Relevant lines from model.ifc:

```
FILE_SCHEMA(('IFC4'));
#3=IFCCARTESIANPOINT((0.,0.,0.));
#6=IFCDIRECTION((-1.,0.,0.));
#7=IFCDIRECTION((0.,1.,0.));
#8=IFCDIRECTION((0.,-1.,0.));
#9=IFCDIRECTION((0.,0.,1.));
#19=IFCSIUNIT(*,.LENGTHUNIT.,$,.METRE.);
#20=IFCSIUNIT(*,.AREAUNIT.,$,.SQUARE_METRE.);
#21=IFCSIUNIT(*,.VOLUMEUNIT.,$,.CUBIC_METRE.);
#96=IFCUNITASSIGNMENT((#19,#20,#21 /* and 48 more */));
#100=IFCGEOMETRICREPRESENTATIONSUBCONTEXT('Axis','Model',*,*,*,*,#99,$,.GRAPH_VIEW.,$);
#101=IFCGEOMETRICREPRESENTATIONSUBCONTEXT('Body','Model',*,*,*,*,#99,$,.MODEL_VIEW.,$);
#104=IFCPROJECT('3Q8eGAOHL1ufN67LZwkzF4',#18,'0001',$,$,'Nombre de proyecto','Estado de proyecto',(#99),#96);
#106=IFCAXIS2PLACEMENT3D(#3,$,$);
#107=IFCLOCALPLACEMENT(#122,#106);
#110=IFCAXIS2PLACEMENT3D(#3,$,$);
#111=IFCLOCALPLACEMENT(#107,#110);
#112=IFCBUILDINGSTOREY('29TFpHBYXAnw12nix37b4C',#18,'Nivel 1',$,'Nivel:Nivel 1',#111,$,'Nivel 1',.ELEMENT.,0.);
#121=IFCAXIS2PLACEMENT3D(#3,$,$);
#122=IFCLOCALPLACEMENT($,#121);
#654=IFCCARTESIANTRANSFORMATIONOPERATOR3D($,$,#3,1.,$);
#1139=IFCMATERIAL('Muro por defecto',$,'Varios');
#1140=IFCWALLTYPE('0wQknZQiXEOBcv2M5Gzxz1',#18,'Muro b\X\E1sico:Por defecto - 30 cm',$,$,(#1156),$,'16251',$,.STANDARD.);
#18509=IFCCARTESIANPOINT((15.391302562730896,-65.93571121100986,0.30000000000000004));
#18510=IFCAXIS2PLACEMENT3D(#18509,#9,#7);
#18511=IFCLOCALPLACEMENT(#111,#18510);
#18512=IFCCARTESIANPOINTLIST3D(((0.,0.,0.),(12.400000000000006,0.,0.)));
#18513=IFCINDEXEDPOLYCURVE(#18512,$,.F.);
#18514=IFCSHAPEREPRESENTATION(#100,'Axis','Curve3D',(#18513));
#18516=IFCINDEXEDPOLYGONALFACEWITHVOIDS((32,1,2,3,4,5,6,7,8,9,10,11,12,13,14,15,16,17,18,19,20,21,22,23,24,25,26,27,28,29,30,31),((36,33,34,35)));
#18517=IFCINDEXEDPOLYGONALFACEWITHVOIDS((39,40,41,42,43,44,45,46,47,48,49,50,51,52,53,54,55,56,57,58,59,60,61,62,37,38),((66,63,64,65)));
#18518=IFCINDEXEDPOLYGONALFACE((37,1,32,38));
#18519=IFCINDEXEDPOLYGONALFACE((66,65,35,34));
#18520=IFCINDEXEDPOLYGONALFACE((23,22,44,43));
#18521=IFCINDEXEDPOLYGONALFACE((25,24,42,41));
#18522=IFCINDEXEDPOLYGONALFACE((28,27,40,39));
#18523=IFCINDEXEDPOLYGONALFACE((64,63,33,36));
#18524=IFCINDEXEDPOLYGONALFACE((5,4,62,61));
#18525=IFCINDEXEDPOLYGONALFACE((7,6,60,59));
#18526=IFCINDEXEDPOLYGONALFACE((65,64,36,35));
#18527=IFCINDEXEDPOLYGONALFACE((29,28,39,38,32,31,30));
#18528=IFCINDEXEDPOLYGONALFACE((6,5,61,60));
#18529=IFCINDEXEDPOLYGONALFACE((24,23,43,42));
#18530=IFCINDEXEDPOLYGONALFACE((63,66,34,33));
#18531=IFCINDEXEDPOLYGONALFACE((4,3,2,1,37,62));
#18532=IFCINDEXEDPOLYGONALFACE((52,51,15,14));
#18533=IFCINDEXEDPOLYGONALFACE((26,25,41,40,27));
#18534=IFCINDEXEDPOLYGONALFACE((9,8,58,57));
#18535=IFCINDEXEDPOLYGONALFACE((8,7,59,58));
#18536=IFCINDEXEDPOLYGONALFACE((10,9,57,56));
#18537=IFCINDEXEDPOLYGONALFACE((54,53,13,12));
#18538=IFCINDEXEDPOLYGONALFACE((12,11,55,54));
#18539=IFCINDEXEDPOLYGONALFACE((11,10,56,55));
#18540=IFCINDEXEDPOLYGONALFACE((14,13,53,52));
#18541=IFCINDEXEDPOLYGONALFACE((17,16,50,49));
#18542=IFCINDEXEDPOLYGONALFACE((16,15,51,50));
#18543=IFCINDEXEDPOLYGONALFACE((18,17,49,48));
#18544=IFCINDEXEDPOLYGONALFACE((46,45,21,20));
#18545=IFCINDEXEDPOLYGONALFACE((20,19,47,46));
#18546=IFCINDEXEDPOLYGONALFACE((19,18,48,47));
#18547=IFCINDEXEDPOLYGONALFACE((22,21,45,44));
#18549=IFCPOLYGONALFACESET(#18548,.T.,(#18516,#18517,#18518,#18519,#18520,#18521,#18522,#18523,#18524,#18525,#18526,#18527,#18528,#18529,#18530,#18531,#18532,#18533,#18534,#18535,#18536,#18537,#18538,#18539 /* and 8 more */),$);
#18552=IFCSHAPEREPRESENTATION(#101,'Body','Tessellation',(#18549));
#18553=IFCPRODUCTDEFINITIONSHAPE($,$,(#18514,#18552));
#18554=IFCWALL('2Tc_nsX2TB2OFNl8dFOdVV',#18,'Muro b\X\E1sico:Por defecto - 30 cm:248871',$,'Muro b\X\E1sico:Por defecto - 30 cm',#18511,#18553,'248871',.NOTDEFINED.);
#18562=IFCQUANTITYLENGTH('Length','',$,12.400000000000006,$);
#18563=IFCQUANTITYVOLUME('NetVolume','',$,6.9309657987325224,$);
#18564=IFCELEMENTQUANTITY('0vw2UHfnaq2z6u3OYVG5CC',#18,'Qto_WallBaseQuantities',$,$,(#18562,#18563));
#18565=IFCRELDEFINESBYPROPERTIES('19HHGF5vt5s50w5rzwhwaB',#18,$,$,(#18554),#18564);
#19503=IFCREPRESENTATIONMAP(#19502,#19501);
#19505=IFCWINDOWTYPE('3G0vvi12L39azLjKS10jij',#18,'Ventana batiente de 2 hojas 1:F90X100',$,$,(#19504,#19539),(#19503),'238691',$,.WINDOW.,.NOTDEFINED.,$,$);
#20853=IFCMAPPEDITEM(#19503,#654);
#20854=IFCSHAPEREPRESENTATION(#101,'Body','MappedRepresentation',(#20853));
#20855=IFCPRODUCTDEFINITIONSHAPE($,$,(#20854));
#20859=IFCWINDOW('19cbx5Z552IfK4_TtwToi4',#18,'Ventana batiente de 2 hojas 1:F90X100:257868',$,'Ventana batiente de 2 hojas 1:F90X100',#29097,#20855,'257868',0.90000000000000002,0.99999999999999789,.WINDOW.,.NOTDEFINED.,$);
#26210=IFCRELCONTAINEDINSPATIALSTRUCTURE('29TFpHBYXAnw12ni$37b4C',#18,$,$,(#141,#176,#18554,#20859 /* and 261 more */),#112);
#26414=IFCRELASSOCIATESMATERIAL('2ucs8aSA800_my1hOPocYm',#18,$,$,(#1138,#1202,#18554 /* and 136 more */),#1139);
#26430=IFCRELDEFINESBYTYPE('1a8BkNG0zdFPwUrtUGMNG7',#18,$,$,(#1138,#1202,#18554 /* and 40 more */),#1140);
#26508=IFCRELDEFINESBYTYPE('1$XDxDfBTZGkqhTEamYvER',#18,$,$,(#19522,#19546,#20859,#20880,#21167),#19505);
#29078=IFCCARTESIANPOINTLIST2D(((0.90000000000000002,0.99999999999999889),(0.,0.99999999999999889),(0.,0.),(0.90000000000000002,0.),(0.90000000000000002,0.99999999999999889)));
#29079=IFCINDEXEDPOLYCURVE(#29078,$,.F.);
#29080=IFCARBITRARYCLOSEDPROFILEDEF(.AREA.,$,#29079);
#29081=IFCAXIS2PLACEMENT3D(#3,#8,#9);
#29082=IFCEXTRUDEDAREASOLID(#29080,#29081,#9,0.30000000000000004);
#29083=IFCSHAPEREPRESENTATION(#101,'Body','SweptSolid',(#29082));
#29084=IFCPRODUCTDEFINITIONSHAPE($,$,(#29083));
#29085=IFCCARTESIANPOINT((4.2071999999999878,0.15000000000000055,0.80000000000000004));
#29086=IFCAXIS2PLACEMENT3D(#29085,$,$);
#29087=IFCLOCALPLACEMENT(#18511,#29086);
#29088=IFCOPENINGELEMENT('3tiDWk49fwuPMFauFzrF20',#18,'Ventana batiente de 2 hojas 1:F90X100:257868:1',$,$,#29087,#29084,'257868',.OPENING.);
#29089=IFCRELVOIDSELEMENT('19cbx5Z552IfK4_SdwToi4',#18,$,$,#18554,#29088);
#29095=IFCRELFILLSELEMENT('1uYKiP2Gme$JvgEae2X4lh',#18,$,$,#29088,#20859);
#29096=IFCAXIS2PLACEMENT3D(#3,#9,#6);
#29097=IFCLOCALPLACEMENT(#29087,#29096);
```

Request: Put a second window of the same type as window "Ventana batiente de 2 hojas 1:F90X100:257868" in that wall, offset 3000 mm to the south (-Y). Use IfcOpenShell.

```python
import ifcopenshell
import ifcopenshell.api.feature
import ifcopenshell.api.geometry
import ifcopenshell.api.pset
import ifcopenshell.api.root
import ifcopenshell.geom
import ifcopenshell.util.element
import ifcopenshell.util.placement
import ifcopenshell.util.shape
import ifcopenshell.util.unit

model = ifcopenshell.open("model.ifc")
unit_scale = ifcopenshell.util.unit.calculate_unit_scale(model)
volume_scale = ifcopenshell.util.unit.calculate_unit_scale(model, "VOLUMEUNIT")
settings = ifcopenshell.geom.settings()


def volume(element):
    """Net volume in cubic metres, openings subtracted."""
    shape = ifcopenshell.geom.create_shape(settings, element)
    return ifcopenshell.util.shape.get_volume(shape.geometry)


def reuse_history(source, copy):
    """copy_class also copies each property set's owner history, people and application; keep the originals."""
    for rel in copy.IsDefinedBy:
        if rel.is_a("IfcRelDefinesByProperties") and (history := rel.RelatingPropertyDefinition.OwnerHistory):
            rel.RelatingPropertyDefinition.OwnerHistory = source.OwnerHistory
            ifcopenshell.util.element.remove_deep2(model, history)


window = model.by_id(20859)
opening = window.FillsVoids[0].RelatingOpeningElement
wall = opening.VoidsElements[0].RelatingBuildingElement
before = volume(wall)
shift = ifcopenshell.util.placement.get_local_placement(wall.ObjectPlacement)[:3, 0] * -3 / unit_scale

# copy_class copies the void relationship, type, container and properties, but no geometry.
new_opening = ifcopenshell.api.root.copy_class(model, product=opening)
new_opening.Representation = ifcopenshell.util.element.copy_deep(
    model, opening.Representation, exclude=["IfcGeometricRepresentationContext", "IfcRepresentationMap"]
)
new_opening.Name = "Ventana batiente de 2 hojas 1:F90X100"
new_opening.Tag = None
reuse_history(opening, new_opening)
new_window = ifcopenshell.api.root.copy_class(model, product=window)
new_window.Representation = ifcopenshell.util.element.copy_deep(
    model, window.Representation, exclude=["IfcGeometricRepresentationContext", "IfcRepresentationMap"]
)
new_window.Name = "Ventana batiente de 2 hojas 1:F90X100"
new_window.Tag = None
reuse_history(window, new_window)
ifcopenshell.api.feature.add_filling(model, opening=new_opening, element=new_window)

for old, new in ((opening, new_opening), (window, new_window)):
    matrix = ifcopenshell.util.placement.get_local_placement(old.ObjectPlacement)
    matrix[:3, 3] += shift
    ifcopenshell.api.geometry.edit_object_placement(model, product=new, matrix=matrix, is_si=False)

after = volume(wall)

# Update the wall's stored quantities.
qto = model.by_id(ifcopenshell.util.element.get_pset(wall, "Qto_WallBaseQuantities", should_inherit=False)["id"])
ifcopenshell.api.pset.edit_qto(model, qto=qto, properties={"NetVolume": after / volume_scale})

print(f"wall volume {before:.3f} -> {after:.3f} m3")

model.write("model-out.ifc")
```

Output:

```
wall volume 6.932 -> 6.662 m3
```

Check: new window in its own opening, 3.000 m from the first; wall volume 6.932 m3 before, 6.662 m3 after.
